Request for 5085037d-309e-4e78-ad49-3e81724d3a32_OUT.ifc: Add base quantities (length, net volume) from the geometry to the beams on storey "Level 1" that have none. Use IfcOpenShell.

First a look at what the model holds.

```python
import ifcopenshell
import ifcopenshell.util.element
import ifcopenshell.util.unit

model = ifcopenshell.open("5085037d-309e-4e78-ad49-3e81724d3a32_OUT.ifc")
print(model.schema)
for unit_type in ("LENGTHUNIT", "AREAUNIT", "VOLUMEUNIT"):
    print(unit_type, ifcopenshell.util.unit.calculate_unit_scale(model, unit_type))
storey = next(s for s in model.by_type("IfcBuildingStorey") if s.Name == "Level 1")
beams = [e for e in ifcopenshell.util.element.get_decomposition(storey) if e.is_a("IfcBeam")]
for e in sorted(beams, key=lambda e: e.id()):
    print(e.id(), e.is_a(), e.Name, list(ifcopenshell.util.element.get_psets(e, qtos_only=True)), sep=" | ")
```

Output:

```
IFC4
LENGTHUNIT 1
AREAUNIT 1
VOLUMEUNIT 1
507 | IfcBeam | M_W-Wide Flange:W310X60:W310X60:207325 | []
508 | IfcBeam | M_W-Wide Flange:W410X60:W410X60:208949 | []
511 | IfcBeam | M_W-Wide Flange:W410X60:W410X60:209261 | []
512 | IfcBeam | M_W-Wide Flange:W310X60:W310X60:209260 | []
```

```python
import ifcopenshell
import ifcopenshell.api.pset
import ifcopenshell.geom
import ifcopenshell.util.element
import ifcopenshell.util.shape
import ifcopenshell.util.unit

model = ifcopenshell.open("5085037d-309e-4e78-ad49-3e81724d3a32_OUT.ifc")
unit_scale = ifcopenshell.util.unit.calculate_unit_scale(model)
volume_scale = ifcopenshell.util.unit.calculate_unit_scale(model, "VOLUMEUNIT")
settings = ifcopenshell.geom.settings()

storey = next(s for s in model.by_type("IfcBuildingStorey") if s.Name == "Level 1")
beams = [e for e in ifcopenshell.util.element.get_decomposition(storey) if e.is_a("IfcBeam")]

for e in sorted(beams, key=lambda e: e.id()):
    if ifcopenshell.util.element.get_psets(e, qtos_only=True, should_inherit=False):
        continue
    # Geometry comes back in metres, in the element's own axes.
    shape = ifcopenshell.geom.create_shape(settings, e)
    values = {
        "Length": ifcopenshell.util.shape.get_max_xyz(shape.geometry) / unit_scale,
        "NetVolume": ifcopenshell.util.shape.get_volume(shape.geometry) / volume_scale,
    }
    qto = ifcopenshell.api.pset.add_qto(model, product=e, name="Qto_BeamBaseQuantities")
    ifcopenshell.api.pset.edit_qto(model, qto=qto, properties=values)
    print(e.id(), {k: round(v, 3) for k, v in values.items()})

model.write("5085037d-309e-4e78-ad49-3e81724d3a32_OUT_rev.ifc")
```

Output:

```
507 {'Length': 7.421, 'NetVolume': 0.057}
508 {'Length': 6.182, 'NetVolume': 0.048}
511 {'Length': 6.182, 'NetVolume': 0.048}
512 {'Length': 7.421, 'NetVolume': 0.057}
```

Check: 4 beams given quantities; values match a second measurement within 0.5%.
